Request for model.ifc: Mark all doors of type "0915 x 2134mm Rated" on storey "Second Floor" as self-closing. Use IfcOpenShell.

First a look at what the model holds.

```python
import ifcopenshell
import ifcopenshell.util.element

model = ifcopenshell.open("model.ifc")
print(model.schema)
storey = next(s for s in model.by_type("IfcBuildingStorey") if s.Name == "Second Floor")
doors = [e for e in ifcopenshell.util.element.get_decomposition(storey) if e.is_a("IfcDoor")]
seen = {}
for e in doors:
    element_type = ifcopenshell.util.element.get_type(e)
    key = (element_type.Name if element_type != e and element_type else None, ifcopenshell.util.element.get_pset(e, "Pset_DoorCommon", "SelfClosing"))
    seen[key] = seen.get(key, 0) + 1
for (name, value), count in sorted(seen.items(), key=str):
    print(count, "x", name, "|", value)
```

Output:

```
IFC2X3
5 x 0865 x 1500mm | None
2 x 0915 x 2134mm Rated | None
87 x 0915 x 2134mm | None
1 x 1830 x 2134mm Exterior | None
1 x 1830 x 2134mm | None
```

```python
import ifcopenshell
import ifcopenshell.api.pset
import ifcopenshell.util.element

model = ifcopenshell.open("model.ifc")

storey = next(s for s in model.by_type("IfcBuildingStorey") if s.Name == "Second Floor")
doors = [e for e in ifcopenshell.util.element.get_decomposition(storey) if e.is_a("IfcDoor")]

count = 0
for e in doors:
    element_type = ifcopenshell.util.element.get_type(e)
    if element_type in (None, e) or element_type.Name != "0915 x 2134mm Rated":
        continue
    # add_pset returns the element's existing set when there is one.
    pset = ifcopenshell.api.pset.add_pset(model, product=e, name="Pset_DoorCommon")
    ifcopenshell.api.pset.edit_pset(model, pset=pset, properties={"SelfClosing": True})
    count += 1

print(count, "doors updated")

model.write("model_rev.ifc")
```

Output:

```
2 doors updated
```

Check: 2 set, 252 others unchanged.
